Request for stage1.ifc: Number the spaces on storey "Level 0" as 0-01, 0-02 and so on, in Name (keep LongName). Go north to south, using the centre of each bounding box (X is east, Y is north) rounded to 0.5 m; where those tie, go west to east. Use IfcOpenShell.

First a look at what the model holds.

```python
import ifcopenshell
import ifcopenshell.util.element
import ifcopenshell.util.placement

model = ifcopenshell.open("stage1.ifc")
print(model.schema)
storey = next(s for s in model.by_type("IfcBuildingStorey") if s.Name == "Level 0")
spaces = [e for e in ifcopenshell.util.element.get_decomposition(storey) if e.is_a("IfcSpace")]
for e in sorted(spaces, key=lambda e: e.id()):
    origin = ifcopenshell.util.placement.get_local_placement(e.ObjectPlacement)[:3, 3]
    print(e.id(), e.Name, e.LongName, origin.round(2) + 0.0, sep=" | ")
```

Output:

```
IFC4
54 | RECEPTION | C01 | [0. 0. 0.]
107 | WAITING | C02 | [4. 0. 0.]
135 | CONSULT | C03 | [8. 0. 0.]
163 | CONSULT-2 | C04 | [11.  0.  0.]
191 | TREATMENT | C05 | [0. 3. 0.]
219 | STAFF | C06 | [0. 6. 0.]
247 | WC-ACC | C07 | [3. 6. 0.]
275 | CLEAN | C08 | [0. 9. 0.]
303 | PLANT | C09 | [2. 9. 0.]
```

```python
import ifcopenshell
import ifcopenshell.geom
import ifcopenshell.util.element
import ifcopenshell.util.shape

model = ifcopenshell.open("stage1.ifc")
settings = ifcopenshell.geom.settings()
settings.set("use-world-coords", True)


def centre(element):
    shape = ifcopenshell.geom.create_shape(settings, element)
    return ifcopenshell.util.shape.get_bbox_centroid(shape.geometry)


storey = next(s for s in model.by_type("IfcBuildingStorey") if s.Name == "Level 0")
spaces = [e for e in ifcopenshell.util.element.get_decomposition(storey) if e.is_a("IfcSpace")]

# Insertion points can sit at a corner or the storey origin, so sort by the geometry (in metres).
centres = {e: centre(e) for e in spaces}
spaces.sort(key=lambda e: (-round(centres[e][1] / 0.5), centres[e][0]))

for i, e in enumerate(spaces, start=1):
    number = f"0-{i:02d}"
    e.Name = number
    print(e.id(), number)

model.write("stage1_rev.ifc")
```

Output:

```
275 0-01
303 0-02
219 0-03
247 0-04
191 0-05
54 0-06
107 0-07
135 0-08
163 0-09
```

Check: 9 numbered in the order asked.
